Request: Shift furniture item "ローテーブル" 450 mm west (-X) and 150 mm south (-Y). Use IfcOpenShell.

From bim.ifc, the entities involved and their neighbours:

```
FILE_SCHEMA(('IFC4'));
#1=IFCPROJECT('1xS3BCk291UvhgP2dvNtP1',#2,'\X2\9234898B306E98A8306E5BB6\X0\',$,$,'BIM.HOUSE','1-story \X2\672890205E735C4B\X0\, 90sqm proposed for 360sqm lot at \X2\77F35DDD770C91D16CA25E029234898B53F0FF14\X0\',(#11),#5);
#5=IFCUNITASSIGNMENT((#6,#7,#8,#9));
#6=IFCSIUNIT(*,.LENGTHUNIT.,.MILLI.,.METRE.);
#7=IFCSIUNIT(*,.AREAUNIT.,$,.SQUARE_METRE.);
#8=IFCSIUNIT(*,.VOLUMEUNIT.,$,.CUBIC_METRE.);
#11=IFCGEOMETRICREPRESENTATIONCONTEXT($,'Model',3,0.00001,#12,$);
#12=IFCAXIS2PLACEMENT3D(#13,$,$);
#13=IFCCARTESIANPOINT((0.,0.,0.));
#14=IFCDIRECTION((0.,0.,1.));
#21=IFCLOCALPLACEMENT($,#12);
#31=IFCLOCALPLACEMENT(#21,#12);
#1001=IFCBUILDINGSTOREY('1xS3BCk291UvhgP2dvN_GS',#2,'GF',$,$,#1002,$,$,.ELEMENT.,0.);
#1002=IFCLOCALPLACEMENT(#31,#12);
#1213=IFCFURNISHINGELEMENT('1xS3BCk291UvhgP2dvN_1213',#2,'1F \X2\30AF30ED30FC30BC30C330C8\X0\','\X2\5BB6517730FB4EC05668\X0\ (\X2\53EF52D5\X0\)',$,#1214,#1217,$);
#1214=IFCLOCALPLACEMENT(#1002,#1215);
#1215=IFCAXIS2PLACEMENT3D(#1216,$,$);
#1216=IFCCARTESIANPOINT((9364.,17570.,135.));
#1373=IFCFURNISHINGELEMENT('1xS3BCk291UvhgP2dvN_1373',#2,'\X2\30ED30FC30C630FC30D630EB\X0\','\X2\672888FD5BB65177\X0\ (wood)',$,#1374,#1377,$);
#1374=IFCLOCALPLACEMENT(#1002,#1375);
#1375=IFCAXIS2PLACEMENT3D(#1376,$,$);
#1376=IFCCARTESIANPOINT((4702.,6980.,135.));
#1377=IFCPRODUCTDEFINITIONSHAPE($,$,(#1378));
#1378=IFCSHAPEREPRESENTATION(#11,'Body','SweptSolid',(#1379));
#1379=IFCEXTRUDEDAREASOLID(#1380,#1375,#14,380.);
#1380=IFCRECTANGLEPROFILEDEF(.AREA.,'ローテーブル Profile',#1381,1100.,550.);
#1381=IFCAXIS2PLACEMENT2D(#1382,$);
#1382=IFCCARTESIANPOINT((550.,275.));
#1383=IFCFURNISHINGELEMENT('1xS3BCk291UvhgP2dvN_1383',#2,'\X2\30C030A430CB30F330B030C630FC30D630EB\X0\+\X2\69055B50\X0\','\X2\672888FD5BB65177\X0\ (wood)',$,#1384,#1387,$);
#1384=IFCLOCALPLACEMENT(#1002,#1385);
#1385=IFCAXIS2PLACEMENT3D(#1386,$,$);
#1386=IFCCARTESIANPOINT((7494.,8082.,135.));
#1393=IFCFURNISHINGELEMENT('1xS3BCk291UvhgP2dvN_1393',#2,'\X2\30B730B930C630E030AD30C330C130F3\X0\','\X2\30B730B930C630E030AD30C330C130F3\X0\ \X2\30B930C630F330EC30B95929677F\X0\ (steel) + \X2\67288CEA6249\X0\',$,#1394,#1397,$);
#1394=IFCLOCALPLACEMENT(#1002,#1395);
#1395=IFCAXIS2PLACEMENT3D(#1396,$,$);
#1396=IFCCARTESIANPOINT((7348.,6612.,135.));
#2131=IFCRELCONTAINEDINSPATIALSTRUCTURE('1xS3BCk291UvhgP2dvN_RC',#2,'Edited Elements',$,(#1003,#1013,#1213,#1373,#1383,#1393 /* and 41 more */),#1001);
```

```python
import ifcopenshell
import ifcopenshell.api.geometry
import ifcopenshell.util.placement
import ifcopenshell.util.unit

model = ifcopenshell.open("bim.ifc")
unit_scale = ifcopenshell.util.unit.calculate_unit_scale(model)

item = model.by_id(1373)
matrix = ifcopenshell.util.placement.get_local_placement(item.ObjectPlacement)
matrix[0, 3] -= 0.45 / unit_scale
matrix[1, 3] -= 0.15 / unit_scale
ifcopenshell.api.geometry.edit_object_placement(model, product=item, matrix=matrix, is_si=False)

print(ifcopenshell.util.placement.get_local_placement(item.ObjectPlacement).round(3) + 0.0)

model.write("bim_rev.ifc")
```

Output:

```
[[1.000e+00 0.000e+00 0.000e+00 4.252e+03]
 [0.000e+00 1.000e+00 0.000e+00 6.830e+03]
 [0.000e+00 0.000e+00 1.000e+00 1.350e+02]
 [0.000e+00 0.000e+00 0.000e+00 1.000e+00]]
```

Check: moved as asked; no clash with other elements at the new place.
